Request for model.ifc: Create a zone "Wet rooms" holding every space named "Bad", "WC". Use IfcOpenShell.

First a look at what the model holds.

```python
import ifcopenshell

model = ifcopenshell.open("model.ifc")
print(model.schema)
seen = {}
for space in model.by_type("IfcSpace"):
    seen[space.LongName] = seen.get(space.LongName, 0) + 1
for name, count in sorted(seen.items(), key=str):
    print(count, "x", name)
print("zones:", [z.Name for z in model.by_type("IfcZone")][:20])
```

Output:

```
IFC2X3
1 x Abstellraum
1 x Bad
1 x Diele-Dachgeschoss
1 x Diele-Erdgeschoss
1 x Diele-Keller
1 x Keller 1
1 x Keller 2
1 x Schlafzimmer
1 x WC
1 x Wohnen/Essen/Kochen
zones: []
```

```python
import ifcopenshell
import ifcopenshell.api.group
import ifcopenshell.api.root

model = ifcopenshell.open("model.ifc")

names = {"Bad", "WC"}
spaces = [s for s in model.by_type("IfcSpace") if s.LongName in names]

zone = ifcopenshell.api.root.create_entity(model, ifc_class="IfcZone", name="Wet rooms")
ifcopenshell.api.group.assign_group(model, products=spaces, group=zone)
print(len(spaces), "spaces in", zone.Name)

model.write("model_v2.ifc")
```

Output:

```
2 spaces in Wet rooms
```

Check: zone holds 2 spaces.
